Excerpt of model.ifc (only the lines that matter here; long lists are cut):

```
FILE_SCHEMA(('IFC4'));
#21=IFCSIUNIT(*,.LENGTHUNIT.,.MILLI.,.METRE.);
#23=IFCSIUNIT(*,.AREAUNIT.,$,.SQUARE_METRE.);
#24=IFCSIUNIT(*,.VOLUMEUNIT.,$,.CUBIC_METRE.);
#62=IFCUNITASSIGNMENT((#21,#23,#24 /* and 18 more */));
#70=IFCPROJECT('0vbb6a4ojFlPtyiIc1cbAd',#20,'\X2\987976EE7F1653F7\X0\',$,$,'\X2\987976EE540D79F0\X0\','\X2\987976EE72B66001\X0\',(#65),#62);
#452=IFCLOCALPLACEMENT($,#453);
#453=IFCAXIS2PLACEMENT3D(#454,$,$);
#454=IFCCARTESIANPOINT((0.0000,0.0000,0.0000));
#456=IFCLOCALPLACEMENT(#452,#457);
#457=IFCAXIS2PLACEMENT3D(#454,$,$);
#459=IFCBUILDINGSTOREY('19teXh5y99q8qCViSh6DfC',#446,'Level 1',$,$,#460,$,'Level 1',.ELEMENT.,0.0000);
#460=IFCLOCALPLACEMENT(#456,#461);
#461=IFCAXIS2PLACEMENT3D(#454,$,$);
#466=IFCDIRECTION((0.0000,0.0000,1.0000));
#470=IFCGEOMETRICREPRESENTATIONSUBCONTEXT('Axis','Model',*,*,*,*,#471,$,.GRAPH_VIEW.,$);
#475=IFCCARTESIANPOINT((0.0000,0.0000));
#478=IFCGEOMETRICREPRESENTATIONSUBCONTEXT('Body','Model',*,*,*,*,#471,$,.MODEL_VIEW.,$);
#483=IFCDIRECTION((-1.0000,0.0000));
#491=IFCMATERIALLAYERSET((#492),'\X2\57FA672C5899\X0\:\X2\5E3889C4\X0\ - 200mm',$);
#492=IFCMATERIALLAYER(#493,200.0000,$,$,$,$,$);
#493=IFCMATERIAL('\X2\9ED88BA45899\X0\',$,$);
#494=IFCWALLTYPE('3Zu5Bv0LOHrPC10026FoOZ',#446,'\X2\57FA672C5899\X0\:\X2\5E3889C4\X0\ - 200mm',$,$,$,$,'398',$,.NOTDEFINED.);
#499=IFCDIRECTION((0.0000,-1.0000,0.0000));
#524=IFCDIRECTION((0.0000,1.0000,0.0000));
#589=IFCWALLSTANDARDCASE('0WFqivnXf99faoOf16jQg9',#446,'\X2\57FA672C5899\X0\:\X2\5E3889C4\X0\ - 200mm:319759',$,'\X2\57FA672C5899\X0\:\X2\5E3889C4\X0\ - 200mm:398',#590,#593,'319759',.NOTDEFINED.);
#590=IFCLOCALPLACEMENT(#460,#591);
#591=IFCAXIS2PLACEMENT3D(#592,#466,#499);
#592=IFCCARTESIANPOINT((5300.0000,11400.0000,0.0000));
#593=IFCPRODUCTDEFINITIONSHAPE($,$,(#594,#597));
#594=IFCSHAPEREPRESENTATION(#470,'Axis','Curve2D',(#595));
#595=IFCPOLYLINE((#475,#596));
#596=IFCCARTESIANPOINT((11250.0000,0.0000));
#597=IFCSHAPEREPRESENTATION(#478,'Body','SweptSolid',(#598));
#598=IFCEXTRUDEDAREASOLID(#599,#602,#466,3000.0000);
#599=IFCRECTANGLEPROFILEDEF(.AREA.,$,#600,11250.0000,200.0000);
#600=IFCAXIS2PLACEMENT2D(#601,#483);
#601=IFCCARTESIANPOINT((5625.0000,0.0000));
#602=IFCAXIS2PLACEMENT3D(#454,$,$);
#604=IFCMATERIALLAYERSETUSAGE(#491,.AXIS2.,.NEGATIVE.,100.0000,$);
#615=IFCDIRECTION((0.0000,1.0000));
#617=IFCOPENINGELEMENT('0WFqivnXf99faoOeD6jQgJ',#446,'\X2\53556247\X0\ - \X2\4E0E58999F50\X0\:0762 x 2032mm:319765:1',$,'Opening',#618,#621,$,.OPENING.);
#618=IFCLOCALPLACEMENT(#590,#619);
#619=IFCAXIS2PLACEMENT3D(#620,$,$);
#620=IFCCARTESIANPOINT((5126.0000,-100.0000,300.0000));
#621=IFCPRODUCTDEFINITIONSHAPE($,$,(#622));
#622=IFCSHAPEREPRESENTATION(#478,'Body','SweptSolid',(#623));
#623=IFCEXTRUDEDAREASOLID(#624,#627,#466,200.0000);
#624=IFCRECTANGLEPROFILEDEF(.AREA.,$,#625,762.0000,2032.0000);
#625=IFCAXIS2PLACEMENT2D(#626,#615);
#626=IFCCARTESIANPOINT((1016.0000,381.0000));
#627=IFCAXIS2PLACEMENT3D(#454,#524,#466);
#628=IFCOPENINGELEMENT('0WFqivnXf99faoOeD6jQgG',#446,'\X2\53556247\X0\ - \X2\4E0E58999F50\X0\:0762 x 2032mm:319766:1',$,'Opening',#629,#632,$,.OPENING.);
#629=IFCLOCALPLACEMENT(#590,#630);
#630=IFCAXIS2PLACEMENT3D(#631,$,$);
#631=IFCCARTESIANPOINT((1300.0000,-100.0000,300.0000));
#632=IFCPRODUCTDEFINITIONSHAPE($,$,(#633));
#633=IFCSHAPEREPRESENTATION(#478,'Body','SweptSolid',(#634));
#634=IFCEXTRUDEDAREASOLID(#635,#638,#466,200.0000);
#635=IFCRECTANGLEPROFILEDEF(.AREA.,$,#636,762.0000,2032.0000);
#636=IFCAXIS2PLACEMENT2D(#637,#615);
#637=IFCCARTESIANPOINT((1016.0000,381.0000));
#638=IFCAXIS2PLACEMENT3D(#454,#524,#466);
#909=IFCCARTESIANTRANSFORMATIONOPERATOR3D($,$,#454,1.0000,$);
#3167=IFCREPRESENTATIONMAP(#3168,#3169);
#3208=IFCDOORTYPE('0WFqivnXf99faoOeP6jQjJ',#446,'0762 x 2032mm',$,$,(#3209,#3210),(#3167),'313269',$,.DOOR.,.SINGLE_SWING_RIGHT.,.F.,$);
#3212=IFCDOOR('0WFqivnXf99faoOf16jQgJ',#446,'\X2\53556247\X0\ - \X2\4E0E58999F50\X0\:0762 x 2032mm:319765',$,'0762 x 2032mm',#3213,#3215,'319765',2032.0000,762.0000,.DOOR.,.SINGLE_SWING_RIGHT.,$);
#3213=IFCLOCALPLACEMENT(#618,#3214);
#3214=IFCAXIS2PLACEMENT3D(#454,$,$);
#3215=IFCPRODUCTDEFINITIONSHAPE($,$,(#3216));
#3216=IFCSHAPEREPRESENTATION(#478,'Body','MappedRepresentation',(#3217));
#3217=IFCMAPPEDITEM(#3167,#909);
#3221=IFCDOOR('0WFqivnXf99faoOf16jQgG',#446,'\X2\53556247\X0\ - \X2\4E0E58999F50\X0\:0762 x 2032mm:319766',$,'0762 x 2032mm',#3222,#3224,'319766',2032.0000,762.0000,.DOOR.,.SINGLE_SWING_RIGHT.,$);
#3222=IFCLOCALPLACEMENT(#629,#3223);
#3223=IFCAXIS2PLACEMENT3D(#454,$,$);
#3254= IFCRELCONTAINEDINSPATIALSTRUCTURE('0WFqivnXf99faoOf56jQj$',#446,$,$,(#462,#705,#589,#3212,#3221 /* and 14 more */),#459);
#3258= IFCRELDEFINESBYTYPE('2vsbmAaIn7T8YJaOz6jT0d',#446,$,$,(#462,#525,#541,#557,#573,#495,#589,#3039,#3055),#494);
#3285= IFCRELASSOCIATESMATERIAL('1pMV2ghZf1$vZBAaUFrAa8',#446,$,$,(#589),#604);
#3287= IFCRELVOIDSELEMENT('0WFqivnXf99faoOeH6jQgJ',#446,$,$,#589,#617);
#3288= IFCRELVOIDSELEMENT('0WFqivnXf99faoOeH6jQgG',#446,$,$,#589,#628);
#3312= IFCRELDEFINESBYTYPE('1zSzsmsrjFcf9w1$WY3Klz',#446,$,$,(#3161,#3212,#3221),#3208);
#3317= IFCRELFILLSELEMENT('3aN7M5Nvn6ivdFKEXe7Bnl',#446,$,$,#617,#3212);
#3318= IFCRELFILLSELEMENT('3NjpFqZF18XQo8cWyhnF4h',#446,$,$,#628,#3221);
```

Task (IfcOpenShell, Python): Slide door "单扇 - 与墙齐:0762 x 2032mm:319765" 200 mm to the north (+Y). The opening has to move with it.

```python
import ifcopenshell
import ifcopenshell.api.geometry
import ifcopenshell.util.placement
import ifcopenshell.util.unit

model = ifcopenshell.open("model.ifc")
unit_scale = ifcopenshell.util.unit.calculate_unit_scale(model)

door = model.by_guid("0WFqivnXf99faoOf16jQgJ")
opening = door.FillsVoids[0].RelatingOpeningElement
wall = opening.VoidsElements[0].RelatingBuildingElement

wall_matrix = ifcopenshell.util.placement.get_local_placement(wall.ObjectPlacement)
shift = wall_matrix[:3, 0] * -0.2 / unit_scale
before = ifcopenshell.util.placement.get_local_placement(door.ObjectPlacement)[:3, 3].copy()

# The door is placed relative to its opening, so it follows when the opening moves.
matrix = ifcopenshell.util.placement.get_local_placement(opening.ObjectPlacement)
matrix[:3, 3] += shift
ifcopenshell.api.geometry.edit_object_placement(
    model, product=opening, matrix=matrix, is_si=False, should_transform_children=True
)

after = ifcopenshell.util.placement.get_local_placement(door.ObjectPlacement)[:3, 3]
print("door moved by", (after - before).round(3) + 0.0)

model.write("model_updated.ifc")
```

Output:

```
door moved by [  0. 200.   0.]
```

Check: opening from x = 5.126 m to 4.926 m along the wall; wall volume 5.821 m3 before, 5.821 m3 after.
